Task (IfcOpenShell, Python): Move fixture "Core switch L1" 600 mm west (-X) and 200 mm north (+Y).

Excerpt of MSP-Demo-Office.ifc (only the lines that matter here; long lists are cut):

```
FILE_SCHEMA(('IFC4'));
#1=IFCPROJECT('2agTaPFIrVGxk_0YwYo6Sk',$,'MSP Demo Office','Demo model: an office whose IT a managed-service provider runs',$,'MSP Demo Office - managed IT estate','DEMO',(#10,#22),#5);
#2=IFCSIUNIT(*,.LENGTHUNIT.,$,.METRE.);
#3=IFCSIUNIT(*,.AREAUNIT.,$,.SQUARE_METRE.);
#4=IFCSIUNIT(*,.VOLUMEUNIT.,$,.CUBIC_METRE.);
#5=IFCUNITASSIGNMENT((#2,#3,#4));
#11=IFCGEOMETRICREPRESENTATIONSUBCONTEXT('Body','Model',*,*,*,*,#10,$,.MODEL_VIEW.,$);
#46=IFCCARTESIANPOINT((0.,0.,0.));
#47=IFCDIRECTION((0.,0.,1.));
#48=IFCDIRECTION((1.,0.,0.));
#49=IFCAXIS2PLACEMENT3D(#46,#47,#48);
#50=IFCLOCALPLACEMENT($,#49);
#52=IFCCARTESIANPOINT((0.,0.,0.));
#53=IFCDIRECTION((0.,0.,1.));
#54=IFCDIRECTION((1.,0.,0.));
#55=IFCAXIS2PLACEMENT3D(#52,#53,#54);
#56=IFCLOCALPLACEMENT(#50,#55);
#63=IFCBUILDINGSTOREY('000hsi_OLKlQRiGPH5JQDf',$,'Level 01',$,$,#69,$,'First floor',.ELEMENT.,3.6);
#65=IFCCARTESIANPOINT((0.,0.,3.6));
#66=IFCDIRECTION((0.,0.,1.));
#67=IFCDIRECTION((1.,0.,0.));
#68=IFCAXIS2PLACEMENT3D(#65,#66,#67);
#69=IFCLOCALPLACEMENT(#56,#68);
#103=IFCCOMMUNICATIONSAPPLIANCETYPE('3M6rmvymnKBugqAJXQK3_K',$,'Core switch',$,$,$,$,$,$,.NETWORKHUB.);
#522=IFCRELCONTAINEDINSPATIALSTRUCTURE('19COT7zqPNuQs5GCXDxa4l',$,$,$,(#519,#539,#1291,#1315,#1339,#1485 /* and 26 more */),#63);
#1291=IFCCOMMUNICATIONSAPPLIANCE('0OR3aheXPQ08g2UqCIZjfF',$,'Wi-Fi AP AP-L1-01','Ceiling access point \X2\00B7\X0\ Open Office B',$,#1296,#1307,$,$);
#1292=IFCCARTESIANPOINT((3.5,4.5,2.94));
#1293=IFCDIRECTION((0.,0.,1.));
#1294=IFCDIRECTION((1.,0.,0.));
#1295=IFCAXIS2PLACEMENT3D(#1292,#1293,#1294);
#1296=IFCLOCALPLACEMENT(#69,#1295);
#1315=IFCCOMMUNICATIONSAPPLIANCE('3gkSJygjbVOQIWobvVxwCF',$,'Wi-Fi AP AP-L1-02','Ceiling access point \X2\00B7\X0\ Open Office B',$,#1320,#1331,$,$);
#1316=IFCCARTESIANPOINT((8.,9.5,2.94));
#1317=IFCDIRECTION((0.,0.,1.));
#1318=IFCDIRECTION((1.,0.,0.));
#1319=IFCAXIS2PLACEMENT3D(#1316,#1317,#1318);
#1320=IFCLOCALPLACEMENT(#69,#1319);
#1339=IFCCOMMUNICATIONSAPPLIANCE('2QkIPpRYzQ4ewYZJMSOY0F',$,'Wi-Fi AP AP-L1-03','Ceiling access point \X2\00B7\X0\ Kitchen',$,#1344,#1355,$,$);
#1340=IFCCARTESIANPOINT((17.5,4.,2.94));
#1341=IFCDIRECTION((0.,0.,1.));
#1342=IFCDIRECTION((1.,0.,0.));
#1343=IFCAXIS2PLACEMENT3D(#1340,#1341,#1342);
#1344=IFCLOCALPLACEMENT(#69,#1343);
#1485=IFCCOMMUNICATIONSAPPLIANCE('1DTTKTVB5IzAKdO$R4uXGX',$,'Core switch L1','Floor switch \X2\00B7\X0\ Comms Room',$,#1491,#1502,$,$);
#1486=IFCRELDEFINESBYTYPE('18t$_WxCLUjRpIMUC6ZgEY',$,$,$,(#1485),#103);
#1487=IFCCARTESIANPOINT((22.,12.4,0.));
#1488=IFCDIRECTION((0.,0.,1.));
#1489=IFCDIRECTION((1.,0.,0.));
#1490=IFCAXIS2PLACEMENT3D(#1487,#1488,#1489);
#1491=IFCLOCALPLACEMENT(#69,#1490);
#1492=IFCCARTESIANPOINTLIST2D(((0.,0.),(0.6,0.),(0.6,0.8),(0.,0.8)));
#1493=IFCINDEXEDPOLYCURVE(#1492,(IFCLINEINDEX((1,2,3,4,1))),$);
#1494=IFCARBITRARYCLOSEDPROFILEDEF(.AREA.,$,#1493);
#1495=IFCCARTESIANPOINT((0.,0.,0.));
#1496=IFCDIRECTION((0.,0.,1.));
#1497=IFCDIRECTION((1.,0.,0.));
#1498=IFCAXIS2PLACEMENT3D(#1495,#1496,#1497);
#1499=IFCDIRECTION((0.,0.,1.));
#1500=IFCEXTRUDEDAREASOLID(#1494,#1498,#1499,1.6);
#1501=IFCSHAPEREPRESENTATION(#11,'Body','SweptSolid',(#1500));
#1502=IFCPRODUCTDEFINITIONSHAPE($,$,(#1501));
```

```python
import ifcopenshell
import ifcopenshell.api.geometry
import ifcopenshell.util.placement
import ifcopenshell.util.unit

model = ifcopenshell.open("MSP-Demo-Office.ifc")
unit_scale = ifcopenshell.util.unit.calculate_unit_scale(model)

item = model.by_guid("1DTTKTVB5IzAKdO$R4uXGX")
matrix = ifcopenshell.util.placement.get_local_placement(item.ObjectPlacement)
matrix[0, 3] -= 0.6 / unit_scale
matrix[1, 3] += 0.2 / unit_scale
ifcopenshell.api.geometry.edit_object_placement(model, product=item, matrix=matrix, is_si=False)

print(ifcopenshell.util.placement.get_local_placement(item.ObjectPlacement).round(3) + 0.0)

model.write("MSP-Demo-Office_rev.ifc")
```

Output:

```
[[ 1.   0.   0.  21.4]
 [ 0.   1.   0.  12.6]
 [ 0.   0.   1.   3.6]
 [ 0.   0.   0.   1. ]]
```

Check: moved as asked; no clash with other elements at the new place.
